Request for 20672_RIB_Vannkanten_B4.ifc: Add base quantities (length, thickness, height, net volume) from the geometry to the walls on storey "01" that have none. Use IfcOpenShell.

First a look at what the model holds.

```python
import ifcopenshell
import ifcopenshell.util.element
import ifcopenshell.util.unit

model = ifcopenshell.open("20672_RIB_Vannkanten_B4.ifc")
print(model.schema)
for unit_type in ("LENGTHUNIT", "AREAUNIT", "VOLUMEUNIT"):
    print(unit_type, ifcopenshell.util.unit.calculate_unit_scale(model, unit_type))
storey = next(s for s in model.by_type("IfcBuildingStorey") if s.Name == "01")
walls = [e for e in ifcopenshell.util.element.get_decomposition(storey) if e.is_a("IfcWall")]
for e in sorted(walls, key=lambda e: e.id()):
    print(e.id(), e.is_a(), e.Name, list(ifcopenshell.util.element.get_psets(e, qtos_only=True)), sep=" | ")
```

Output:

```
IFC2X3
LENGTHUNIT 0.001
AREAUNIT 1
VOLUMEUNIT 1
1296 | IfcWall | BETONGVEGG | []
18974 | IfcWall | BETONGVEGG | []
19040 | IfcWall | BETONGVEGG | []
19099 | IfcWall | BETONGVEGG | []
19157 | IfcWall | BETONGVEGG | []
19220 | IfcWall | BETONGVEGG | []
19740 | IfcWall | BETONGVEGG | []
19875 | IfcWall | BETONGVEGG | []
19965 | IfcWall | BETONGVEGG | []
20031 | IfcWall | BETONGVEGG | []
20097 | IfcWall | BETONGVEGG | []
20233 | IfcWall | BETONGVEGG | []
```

```python
import ifcopenshell
import ifcopenshell.api.pset
import ifcopenshell.geom
import ifcopenshell.util.element
import ifcopenshell.util.shape
import ifcopenshell.util.unit

model = ifcopenshell.open("20672_RIB_Vannkanten_B4.ifc")
unit_scale = ifcopenshell.util.unit.calculate_unit_scale(model)
volume_scale = ifcopenshell.util.unit.calculate_unit_scale(model, "VOLUMEUNIT")
settings = ifcopenshell.geom.settings()

storey = next(s for s in model.by_type("IfcBuildingStorey") if s.Name == "01")
walls = [e for e in ifcopenshell.util.element.get_decomposition(storey) if e.is_a("IfcWall")]

for e in sorted(walls, key=lambda e: e.id()):
    if ifcopenshell.util.element.get_psets(e, qtos_only=True, should_inherit=False):
        continue
    # Geometry comes back in metres, in the element's own axes.
    shape = ifcopenshell.geom.create_shape(settings, e)
    values = {
        "Length": ifcopenshell.util.shape.get_x(shape.geometry) / unit_scale,
        "Width": ifcopenshell.util.shape.get_y(shape.geometry) / unit_scale,
        "Height": ifcopenshell.util.shape.get_z(shape.geometry) / unit_scale,
        "NetVolume": ifcopenshell.util.shape.get_volume(shape.geometry) / volume_scale,
    }
    qto = ifcopenshell.api.pset.add_qto(model, product=e, name="BaseQuantities")
    ifcopenshell.api.pset.edit_qto(model, qto=qto, properties=values)
    print(e.id(), {k: round(v, 3) for k, v in values.items()})

model.write("20672_RIB_Vannkanten_B4_v2.ifc")
```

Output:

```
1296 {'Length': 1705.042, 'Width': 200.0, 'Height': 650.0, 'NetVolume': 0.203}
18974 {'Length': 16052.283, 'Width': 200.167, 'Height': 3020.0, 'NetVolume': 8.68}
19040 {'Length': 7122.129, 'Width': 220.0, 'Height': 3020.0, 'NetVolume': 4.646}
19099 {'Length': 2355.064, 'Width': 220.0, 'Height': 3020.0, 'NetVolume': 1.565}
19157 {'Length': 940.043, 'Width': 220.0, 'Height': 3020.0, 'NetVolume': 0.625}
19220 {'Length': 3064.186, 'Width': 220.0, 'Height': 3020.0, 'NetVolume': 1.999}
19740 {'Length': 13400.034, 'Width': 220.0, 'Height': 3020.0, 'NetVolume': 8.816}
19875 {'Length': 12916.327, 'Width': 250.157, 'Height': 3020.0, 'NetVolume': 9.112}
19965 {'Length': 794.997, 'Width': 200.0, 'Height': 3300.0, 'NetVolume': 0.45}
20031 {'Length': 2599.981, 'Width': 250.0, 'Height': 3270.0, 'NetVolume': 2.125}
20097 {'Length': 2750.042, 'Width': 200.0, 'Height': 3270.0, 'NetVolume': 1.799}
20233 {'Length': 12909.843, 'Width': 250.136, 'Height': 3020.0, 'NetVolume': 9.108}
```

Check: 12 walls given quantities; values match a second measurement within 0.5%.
